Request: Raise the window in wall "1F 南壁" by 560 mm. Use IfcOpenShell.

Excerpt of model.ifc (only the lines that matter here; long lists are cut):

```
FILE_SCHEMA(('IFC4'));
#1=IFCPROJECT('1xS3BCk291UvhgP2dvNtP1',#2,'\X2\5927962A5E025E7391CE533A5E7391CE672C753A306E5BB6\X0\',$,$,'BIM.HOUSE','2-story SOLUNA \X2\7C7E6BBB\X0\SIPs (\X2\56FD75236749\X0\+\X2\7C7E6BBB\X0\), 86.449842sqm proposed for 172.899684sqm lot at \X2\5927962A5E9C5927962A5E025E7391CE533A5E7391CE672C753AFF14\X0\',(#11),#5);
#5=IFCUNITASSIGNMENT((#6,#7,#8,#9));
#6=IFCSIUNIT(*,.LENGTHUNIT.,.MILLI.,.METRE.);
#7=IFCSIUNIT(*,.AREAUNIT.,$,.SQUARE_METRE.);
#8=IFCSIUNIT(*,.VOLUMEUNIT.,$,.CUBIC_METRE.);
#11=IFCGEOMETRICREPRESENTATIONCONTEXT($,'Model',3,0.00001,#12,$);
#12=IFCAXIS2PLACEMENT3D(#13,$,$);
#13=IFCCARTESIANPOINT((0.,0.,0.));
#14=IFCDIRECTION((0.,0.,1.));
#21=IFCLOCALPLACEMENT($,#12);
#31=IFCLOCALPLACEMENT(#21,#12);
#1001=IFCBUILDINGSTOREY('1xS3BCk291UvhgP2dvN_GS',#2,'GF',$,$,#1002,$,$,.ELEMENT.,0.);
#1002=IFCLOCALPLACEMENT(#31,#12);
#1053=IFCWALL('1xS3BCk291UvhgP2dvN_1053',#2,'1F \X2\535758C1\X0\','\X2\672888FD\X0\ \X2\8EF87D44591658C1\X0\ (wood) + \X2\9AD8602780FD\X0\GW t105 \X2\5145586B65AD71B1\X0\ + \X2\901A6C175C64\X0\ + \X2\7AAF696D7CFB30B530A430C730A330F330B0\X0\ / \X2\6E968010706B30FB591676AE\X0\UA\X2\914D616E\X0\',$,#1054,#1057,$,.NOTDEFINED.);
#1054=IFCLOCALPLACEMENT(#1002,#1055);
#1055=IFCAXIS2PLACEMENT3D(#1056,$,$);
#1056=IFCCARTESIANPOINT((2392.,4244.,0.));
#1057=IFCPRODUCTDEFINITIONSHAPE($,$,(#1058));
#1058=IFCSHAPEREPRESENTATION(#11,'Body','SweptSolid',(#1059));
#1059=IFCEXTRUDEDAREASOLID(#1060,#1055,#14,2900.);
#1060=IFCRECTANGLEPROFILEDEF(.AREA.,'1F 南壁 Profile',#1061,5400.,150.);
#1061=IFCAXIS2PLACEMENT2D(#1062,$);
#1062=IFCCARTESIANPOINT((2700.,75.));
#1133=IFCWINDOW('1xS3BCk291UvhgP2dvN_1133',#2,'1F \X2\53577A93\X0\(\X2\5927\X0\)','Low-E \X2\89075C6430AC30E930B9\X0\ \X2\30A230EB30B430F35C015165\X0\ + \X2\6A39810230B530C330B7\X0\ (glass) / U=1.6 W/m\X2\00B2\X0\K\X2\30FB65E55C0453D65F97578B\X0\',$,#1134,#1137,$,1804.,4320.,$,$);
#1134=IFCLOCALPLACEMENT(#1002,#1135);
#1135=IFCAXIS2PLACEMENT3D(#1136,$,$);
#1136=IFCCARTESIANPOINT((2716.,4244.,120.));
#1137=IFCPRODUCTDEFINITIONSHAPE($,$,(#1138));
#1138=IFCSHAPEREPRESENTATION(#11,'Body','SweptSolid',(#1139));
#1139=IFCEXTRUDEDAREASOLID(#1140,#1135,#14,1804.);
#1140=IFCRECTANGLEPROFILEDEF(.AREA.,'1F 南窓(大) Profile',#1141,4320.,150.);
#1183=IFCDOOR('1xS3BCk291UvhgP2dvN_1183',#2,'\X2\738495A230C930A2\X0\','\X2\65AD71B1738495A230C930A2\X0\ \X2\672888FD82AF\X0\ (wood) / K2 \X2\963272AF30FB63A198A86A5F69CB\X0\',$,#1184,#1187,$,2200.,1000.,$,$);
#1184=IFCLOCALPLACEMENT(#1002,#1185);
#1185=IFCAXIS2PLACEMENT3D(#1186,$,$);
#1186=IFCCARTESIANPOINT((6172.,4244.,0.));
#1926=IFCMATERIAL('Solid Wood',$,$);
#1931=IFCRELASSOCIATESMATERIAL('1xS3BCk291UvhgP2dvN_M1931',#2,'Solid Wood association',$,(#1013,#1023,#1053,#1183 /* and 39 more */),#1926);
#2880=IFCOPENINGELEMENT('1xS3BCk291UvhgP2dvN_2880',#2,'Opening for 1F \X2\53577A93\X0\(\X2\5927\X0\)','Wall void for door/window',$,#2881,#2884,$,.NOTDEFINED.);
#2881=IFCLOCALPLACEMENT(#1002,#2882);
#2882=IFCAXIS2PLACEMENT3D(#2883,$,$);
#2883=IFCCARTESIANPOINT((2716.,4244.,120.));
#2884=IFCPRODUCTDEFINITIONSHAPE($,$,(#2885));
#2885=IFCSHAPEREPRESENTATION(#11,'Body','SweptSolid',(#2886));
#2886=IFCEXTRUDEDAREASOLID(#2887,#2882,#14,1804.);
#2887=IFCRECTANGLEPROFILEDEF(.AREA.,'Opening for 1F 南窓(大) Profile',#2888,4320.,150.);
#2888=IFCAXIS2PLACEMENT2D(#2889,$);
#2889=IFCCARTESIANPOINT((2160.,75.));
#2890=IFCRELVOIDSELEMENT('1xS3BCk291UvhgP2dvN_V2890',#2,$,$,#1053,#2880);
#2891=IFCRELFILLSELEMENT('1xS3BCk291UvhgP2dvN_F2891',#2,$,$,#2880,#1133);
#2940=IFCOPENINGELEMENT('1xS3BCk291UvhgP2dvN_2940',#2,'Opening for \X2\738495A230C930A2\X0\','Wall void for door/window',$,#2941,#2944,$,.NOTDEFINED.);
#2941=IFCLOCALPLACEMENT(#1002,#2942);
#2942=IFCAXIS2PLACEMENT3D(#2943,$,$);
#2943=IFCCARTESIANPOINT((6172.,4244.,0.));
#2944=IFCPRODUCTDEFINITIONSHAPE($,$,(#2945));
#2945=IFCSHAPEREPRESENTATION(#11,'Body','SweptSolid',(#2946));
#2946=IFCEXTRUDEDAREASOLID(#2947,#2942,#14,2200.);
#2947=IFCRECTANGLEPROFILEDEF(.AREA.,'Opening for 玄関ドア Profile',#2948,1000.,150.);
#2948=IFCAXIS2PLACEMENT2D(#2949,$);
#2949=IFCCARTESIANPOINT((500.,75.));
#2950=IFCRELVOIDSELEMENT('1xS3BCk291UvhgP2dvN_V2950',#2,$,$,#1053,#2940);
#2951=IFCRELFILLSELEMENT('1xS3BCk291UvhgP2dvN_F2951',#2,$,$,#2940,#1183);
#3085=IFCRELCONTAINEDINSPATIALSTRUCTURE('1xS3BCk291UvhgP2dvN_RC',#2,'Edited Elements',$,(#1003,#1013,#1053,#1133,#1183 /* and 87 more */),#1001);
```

```python
import numpy as np
import ifcopenshell
import ifcopenshell.api.geometry
import ifcopenshell.util.placement
import ifcopenshell.util.unit

model = ifcopenshell.open("model.ifc")
unit_scale = ifcopenshell.util.unit.calculate_unit_scale(model)

window = model.by_guid("1xS3BCk291UvhgP2dvN_1133")
opening = window.FillsVoids[0].RelatingOpeningElement
dz = 0.56 / unit_scale

shift = np.array([0.0, 0.0, dz])
# The window is not placed relative to its opening, so move both.
for product in (opening, window):
    matrix = ifcopenshell.util.placement.get_local_placement(product.ObjectPlacement)
    matrix[:3, 3] += shift
    ifcopenshell.api.geometry.edit_object_placement(model, product=product, matrix=matrix, is_si=False)

print(f"moved by {dz * unit_scale:+.3f} m")

model.write("model-out.ifc")
```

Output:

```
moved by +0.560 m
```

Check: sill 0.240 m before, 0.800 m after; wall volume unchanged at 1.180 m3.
